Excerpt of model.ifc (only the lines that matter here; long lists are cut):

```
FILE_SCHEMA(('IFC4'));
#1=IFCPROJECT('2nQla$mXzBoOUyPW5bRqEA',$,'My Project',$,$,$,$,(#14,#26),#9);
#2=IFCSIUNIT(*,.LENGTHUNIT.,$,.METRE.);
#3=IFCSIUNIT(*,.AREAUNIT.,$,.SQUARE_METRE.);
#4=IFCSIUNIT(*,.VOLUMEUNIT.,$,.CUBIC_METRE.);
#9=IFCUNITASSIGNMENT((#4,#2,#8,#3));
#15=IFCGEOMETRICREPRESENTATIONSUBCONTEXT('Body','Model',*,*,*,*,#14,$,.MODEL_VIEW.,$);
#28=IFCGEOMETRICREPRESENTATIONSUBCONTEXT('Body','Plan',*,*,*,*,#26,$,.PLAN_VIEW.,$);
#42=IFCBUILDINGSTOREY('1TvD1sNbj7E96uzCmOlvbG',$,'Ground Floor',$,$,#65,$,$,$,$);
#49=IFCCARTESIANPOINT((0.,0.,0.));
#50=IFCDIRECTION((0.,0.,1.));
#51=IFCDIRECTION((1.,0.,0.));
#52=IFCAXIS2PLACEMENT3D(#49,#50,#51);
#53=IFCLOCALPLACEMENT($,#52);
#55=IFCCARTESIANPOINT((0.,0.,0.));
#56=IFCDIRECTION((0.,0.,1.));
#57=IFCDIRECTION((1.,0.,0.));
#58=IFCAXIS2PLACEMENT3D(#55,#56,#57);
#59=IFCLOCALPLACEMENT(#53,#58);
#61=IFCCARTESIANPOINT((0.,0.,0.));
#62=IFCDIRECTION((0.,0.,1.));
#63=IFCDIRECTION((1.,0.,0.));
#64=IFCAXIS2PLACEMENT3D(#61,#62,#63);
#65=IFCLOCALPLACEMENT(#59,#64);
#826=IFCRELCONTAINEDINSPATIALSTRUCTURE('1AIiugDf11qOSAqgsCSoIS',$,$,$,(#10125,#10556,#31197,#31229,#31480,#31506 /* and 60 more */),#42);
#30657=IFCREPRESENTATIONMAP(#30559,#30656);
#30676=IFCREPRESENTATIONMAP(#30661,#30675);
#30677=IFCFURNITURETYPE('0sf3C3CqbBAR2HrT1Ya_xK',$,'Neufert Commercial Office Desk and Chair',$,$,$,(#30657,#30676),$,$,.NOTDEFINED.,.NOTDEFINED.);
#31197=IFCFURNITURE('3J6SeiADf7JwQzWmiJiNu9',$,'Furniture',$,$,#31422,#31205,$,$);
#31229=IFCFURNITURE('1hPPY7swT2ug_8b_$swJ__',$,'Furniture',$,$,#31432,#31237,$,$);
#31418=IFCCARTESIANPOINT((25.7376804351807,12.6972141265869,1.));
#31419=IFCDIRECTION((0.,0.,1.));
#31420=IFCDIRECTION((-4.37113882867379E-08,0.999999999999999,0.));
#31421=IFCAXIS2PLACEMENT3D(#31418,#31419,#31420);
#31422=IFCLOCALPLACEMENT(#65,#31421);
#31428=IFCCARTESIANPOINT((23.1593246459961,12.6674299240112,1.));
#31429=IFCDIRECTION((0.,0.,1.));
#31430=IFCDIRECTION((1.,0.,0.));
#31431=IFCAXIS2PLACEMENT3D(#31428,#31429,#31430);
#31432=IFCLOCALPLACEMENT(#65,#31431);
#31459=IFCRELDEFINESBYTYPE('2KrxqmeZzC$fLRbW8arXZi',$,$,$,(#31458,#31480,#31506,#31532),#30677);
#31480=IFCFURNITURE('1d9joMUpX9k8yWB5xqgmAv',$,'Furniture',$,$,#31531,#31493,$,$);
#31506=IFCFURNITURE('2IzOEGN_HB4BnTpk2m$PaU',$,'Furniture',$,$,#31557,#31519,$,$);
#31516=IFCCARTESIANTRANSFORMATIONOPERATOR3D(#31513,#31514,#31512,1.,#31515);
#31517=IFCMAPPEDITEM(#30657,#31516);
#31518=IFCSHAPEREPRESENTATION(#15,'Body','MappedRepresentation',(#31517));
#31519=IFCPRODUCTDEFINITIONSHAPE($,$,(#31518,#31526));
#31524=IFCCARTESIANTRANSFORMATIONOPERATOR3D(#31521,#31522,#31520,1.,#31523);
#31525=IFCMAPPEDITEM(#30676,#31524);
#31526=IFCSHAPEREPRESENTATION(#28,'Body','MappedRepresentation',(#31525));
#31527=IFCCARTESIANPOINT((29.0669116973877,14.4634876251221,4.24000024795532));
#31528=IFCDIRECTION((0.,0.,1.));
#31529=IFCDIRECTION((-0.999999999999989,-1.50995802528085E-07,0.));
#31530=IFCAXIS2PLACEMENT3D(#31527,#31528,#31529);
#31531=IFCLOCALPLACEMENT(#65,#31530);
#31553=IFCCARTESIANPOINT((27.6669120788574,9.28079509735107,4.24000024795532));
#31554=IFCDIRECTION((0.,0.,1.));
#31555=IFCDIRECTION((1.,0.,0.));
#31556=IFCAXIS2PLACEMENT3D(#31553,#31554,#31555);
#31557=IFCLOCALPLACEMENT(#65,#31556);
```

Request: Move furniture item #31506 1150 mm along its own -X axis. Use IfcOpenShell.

```python
import ifcopenshell
import ifcopenshell.api.geometry
import ifcopenshell.util.placement
import ifcopenshell.util.unit

model = ifcopenshell.open("model.ifc")
unit_scale = ifcopenshell.util.unit.calculate_unit_scale(model)

item = model.by_id(31506)
matrix = ifcopenshell.util.placement.get_local_placement(item.ObjectPlacement)
matrix[:3, 3] -= matrix[:3, 0] * 1.15 / unit_scale
ifcopenshell.api.geometry.edit_object_placement(model, product=item, matrix=matrix, is_si=False)

print(ifcopenshell.util.placement.get_local_placement(item.ObjectPlacement).round(3) + 0.0)

model.write("model_v2.ifc")
```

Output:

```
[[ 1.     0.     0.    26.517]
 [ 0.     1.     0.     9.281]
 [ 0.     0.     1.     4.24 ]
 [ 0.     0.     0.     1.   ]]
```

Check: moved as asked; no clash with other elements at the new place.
